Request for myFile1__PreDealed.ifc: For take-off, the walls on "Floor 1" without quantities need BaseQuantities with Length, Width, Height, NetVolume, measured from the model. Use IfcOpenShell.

First a look at what the model holds.

```python
import ifcopenshell
import ifcopenshell.util.element
import ifcopenshell.util.unit

model = ifcopenshell.open("myFile1__PreDealed.ifc")
print(model.schema)
for unit_type in ("LENGTHUNIT", "AREAUNIT", "VOLUMEUNIT"):
    print(unit_type, ifcopenshell.util.unit.calculate_unit_scale(model, unit_type))
storey = next(s for s in model.by_type("IfcBuildingStorey") if s.Name == "Floor 1")
walls = [e for e in ifcopenshell.util.element.get_decomposition(storey) if e.is_a("IfcWall")]
for e in sorted(walls, key=lambda e: e.id()):
    print(e.id(), e.is_a(), e.Name, list(ifcopenshell.util.element.get_psets(e, qtos_only=True)), sep=" | ")
```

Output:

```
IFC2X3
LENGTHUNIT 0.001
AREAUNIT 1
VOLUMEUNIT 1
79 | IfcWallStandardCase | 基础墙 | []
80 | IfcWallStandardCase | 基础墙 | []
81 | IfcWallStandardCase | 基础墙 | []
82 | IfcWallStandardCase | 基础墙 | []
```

```python
import ifcopenshell
import ifcopenshell.api.pset
import ifcopenshell.geom
import ifcopenshell.util.element
import ifcopenshell.util.shape
import ifcopenshell.util.unit

model = ifcopenshell.open("myFile1__PreDealed.ifc")
unit_scale = ifcopenshell.util.unit.calculate_unit_scale(model)
volume_scale = ifcopenshell.util.unit.calculate_unit_scale(model, "VOLUMEUNIT")
settings = ifcopenshell.geom.settings()

storey = next(s for s in model.by_type("IfcBuildingStorey") if s.Name == "Floor 1")
walls = [e for e in ifcopenshell.util.element.get_decomposition(storey) if e.is_a("IfcWall")]

for e in sorted(walls, key=lambda e: e.id()):
    if ifcopenshell.util.element.get_psets(e, qtos_only=True, should_inherit=False):
        continue
    # Geometry comes back in metres, in the element's own axes.
    shape = ifcopenshell.geom.create_shape(settings, e)
    values = {
        "Length": ifcopenshell.util.shape.get_x(shape.geometry) / unit_scale,
        "Width": ifcopenshell.util.shape.get_y(shape.geometry) / unit_scale,
        "Height": ifcopenshell.util.shape.get_z(shape.geometry) / unit_scale,
        "NetVolume": ifcopenshell.util.shape.get_volume(shape.geometry) / volume_scale,
    }
    qto = ifcopenshell.api.pset.add_qto(model, product=e, name="BaseQuantities")
    ifcopenshell.api.pset.edit_qto(model, qto=qto, properties=values)
    print(e.id(), {k: round(v, 3) for k, v in values.items()})

model.write("myFile1__PreDealed_updated.ifc")
```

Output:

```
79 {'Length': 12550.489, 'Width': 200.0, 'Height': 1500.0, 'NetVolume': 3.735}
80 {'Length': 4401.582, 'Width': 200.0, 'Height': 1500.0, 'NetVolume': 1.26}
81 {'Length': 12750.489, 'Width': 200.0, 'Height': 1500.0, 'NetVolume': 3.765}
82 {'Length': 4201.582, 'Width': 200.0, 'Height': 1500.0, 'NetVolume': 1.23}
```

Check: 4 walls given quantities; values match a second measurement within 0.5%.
